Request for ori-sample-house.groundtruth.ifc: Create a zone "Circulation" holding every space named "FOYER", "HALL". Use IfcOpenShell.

First a look at what the model holds.

```python
import ifcopenshell

model = ifcopenshell.open("ori-sample-house.groundtruth.ifc")
print(model.schema)
seen = {}
for space in model.by_type("IfcSpace"):
    seen[space.Name] = seen.get(space.Name, 0) + 1
for name, count in sorted(seen.items(), key=str):
    print(count, "x", name)
print("zones:", [z.Name for z in model.by_type("IfcZone")][:20])
```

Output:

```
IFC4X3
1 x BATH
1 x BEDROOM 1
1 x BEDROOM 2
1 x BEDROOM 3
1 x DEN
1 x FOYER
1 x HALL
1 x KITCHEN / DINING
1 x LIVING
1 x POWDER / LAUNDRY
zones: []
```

```python
import ifcopenshell
import ifcopenshell.api.group
import ifcopenshell.api.root

model = ifcopenshell.open("ori-sample-house.groundtruth.ifc")

names = {"FOYER", "HALL"}
spaces = [s for s in model.by_type("IfcSpace") if s.Name in names]

zone = ifcopenshell.api.root.create_entity(model, ifc_class="IfcZone", name="Circulation")
ifcopenshell.api.group.assign_group(model, products=spaces, group=zone)
print(len(spaces), "spaces in", zone.Name)

model.write("ori-sample-house.groundtruth_edited.ifc")
```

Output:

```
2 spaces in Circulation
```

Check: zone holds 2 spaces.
